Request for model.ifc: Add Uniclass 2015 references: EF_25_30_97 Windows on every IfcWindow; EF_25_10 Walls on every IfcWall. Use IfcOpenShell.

First a look at what the model holds.

```python
import ifcopenshell

model = ifcopenshell.open("model.ifc")
print(model.schema)
print("classifications:", [c.Name for c in model.by_type("IfcClassification")])
for ifc_class in ("IfcDoor", "IfcRoof", "IfcStair", "IfcWall", "IfcWindow"):
    print(ifc_class, len(model.by_type(ifc_class)))
```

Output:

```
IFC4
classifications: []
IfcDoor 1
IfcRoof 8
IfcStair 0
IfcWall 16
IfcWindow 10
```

```python
import ifcopenshell
import ifcopenshell.api.classification

model = ifcopenshell.open("model.ifc")

system = ifcopenshell.api.classification.add_classification(model, classification="Uniclass 2015")

codes = {
    "IfcWindow": ("EF_25_30_97", "Windows"),
    "IfcWall": ("EF_25_10", "Walls"),
}
for ifc_class, (code, name) in codes.items():
    products = model.by_type(ifc_class)
    ifcopenshell.api.classification.add_reference(
        model, products=products, classification=system, identification=code, name=name
    )
    print(code, len(products))

model.write("model_updated.ifc")
```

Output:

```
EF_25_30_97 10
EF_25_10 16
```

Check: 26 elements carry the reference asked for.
